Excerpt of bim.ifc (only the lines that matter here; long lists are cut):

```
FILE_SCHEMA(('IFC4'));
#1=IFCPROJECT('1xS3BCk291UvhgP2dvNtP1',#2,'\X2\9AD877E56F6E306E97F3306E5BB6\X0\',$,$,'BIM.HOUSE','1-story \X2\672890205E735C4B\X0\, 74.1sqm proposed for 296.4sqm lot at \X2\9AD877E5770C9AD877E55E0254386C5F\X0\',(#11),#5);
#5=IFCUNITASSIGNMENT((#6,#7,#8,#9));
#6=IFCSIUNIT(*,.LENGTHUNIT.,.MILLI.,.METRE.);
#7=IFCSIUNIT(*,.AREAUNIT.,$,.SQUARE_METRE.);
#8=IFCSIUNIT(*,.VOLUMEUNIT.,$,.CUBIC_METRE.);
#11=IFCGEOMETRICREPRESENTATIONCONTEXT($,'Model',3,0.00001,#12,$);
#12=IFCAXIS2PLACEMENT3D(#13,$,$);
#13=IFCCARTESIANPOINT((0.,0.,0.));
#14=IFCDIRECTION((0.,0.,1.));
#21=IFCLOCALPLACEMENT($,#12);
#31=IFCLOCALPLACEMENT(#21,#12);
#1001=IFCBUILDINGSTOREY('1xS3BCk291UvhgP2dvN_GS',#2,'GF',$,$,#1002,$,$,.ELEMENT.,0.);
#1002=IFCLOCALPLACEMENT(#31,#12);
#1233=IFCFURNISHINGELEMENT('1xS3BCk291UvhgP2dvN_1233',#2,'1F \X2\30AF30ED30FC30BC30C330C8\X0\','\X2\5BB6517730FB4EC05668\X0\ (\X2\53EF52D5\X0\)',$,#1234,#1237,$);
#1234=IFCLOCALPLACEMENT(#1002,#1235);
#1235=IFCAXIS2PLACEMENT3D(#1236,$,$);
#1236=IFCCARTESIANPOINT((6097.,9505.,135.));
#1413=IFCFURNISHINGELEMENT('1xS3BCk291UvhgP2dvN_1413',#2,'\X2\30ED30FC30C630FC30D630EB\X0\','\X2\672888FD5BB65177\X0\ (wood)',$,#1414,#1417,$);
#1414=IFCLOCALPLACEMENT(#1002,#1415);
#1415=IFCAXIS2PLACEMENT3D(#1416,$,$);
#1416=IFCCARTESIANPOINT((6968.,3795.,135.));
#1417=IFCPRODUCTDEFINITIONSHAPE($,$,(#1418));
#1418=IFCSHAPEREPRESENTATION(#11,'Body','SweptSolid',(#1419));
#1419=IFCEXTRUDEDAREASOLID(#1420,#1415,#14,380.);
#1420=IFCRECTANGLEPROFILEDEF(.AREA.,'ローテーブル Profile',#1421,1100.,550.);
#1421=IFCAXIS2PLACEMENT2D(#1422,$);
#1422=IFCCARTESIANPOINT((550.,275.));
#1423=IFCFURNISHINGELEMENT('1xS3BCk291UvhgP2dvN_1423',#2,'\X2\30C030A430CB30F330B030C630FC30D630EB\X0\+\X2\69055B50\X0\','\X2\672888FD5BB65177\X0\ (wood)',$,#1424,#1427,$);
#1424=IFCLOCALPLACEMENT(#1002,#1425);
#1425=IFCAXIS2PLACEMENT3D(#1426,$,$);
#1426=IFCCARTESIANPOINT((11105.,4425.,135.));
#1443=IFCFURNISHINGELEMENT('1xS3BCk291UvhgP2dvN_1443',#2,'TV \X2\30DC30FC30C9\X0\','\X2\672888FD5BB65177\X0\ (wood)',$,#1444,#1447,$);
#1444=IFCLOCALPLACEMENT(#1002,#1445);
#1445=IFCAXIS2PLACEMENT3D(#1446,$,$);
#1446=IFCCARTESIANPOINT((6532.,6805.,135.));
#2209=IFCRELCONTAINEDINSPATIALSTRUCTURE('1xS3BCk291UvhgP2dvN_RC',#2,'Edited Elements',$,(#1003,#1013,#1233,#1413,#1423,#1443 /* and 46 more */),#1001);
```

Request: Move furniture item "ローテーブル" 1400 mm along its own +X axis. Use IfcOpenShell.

```python
import ifcopenshell
import ifcopenshell.api.geometry
import ifcopenshell.util.placement
import ifcopenshell.util.unit

model = ifcopenshell.open("bim.ifc")
unit_scale = ifcopenshell.util.unit.calculate_unit_scale(model)

item = model.by_id(1413)
matrix = ifcopenshell.util.placement.get_local_placement(item.ObjectPlacement)
matrix[:3, 3] += matrix[:3, 0] * 1.4 / unit_scale
ifcopenshell.api.geometry.edit_object_placement(model, product=item, matrix=matrix, is_si=False)

print(ifcopenshell.util.placement.get_local_placement(item.ObjectPlacement).round(3) + 0.0)

model.write("bim_v2.ifc")
```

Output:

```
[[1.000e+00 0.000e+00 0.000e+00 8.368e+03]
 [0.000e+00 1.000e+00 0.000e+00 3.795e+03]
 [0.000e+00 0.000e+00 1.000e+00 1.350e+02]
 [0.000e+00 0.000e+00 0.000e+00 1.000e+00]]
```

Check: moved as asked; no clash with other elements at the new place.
